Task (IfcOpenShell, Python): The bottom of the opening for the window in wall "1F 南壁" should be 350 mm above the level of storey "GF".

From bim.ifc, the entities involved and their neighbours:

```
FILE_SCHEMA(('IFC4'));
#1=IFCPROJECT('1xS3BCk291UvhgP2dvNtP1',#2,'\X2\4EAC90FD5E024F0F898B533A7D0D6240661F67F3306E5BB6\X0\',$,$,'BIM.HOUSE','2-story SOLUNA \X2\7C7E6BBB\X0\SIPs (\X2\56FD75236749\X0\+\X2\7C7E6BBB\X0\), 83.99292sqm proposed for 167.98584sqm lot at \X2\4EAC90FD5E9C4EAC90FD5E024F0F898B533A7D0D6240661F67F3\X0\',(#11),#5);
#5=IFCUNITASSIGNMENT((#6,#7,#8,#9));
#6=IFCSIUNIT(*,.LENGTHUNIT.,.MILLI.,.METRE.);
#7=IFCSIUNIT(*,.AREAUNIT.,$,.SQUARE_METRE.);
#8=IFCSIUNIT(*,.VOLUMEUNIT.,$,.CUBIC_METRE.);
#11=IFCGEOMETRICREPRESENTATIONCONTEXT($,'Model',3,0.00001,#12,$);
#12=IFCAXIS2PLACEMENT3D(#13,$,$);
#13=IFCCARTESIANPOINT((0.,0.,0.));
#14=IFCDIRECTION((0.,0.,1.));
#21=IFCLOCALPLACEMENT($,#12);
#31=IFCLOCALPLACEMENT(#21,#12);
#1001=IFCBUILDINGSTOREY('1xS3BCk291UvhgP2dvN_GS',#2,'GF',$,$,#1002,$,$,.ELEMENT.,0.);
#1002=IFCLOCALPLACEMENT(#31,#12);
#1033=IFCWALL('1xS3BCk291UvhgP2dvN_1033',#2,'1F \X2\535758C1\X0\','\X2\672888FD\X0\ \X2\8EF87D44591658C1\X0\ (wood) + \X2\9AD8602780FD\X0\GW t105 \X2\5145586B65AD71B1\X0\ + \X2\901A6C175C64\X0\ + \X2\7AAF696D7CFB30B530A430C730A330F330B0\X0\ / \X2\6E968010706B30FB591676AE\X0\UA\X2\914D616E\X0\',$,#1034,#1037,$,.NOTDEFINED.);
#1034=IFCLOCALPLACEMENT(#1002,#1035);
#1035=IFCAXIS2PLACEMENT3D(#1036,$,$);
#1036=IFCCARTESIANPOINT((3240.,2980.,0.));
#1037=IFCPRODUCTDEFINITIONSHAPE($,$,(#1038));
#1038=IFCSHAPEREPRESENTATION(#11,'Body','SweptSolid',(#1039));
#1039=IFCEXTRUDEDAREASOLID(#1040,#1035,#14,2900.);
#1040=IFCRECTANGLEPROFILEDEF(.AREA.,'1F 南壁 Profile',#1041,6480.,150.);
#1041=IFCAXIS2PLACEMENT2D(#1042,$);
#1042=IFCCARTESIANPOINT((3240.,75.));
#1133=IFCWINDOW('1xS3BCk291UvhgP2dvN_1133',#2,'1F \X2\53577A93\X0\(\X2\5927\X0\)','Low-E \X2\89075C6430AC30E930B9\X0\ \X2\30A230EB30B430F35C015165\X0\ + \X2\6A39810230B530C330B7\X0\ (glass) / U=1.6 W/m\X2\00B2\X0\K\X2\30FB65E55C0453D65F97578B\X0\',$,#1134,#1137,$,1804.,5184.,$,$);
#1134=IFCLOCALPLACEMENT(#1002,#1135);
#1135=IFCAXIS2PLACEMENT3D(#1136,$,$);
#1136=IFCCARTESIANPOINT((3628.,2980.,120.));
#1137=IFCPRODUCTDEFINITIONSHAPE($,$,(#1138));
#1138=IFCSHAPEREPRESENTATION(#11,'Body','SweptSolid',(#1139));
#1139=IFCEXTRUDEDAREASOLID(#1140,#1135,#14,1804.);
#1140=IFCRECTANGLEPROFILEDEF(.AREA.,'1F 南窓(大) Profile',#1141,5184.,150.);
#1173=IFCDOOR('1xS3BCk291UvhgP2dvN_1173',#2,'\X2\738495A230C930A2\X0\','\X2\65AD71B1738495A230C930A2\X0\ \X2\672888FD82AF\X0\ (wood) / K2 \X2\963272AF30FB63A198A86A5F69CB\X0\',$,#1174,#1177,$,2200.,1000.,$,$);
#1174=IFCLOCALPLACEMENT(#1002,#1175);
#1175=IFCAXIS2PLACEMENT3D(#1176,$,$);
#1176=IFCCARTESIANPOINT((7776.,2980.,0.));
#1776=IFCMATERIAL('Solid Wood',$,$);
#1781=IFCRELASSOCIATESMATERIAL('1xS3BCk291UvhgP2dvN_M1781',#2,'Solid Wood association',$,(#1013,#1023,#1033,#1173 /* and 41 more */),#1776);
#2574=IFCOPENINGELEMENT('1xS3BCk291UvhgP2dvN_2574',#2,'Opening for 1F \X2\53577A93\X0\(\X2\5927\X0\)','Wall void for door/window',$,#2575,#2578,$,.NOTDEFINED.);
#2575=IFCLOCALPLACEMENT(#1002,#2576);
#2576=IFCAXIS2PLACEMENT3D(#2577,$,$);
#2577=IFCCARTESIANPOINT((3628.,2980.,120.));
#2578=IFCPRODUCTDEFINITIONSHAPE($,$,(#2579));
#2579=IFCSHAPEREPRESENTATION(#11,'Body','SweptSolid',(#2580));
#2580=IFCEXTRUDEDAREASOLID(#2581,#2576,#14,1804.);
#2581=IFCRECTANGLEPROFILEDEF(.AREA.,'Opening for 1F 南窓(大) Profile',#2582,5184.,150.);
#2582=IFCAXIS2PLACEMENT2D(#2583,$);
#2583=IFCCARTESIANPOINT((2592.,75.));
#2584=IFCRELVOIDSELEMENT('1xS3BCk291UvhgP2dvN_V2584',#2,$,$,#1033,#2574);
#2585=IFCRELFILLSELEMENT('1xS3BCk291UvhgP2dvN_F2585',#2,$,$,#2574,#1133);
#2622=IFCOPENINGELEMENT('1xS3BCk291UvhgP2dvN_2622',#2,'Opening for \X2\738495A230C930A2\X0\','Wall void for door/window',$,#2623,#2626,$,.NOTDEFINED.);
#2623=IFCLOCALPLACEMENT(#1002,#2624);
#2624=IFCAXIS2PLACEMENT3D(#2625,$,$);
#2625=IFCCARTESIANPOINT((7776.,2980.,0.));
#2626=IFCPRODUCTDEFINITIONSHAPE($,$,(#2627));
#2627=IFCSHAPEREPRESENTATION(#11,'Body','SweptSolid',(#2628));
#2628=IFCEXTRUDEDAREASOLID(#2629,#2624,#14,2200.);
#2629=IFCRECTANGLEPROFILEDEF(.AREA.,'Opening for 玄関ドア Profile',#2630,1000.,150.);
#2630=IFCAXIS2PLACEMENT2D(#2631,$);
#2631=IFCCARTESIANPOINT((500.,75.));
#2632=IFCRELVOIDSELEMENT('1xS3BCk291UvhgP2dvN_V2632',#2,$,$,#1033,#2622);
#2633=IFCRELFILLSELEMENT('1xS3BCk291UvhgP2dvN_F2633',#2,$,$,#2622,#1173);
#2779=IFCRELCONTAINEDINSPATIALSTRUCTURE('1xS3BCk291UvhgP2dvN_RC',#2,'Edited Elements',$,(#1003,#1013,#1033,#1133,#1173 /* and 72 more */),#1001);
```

```python
import numpy as np
import ifcopenshell
import ifcopenshell.api.geometry
import ifcopenshell.geom
import ifcopenshell.util.element
import ifcopenshell.util.placement
import ifcopenshell.util.shape
import ifcopenshell.util.unit

model = ifcopenshell.open("bim.ifc")
unit_scale = ifcopenshell.util.unit.calculate_unit_scale(model)

window = model.by_guid("1xS3BCk291UvhgP2dvN_1133")
opening = window.FillsVoids[0].RelatingOpeningElement
storey = ifcopenshell.util.element.get_container(window, ifc_class="IfcBuildingStorey")
level = ifcopenshell.util.placement.get_local_placement(storey.ObjectPlacement)[2, 3]

# The opening's origin need not be at the sill, so measure its lowest point.
shape = ifcopenshell.geom.create_shape(ifcopenshell.geom.settings(), opening)
bottom = ifcopenshell.util.shape.get_shape_bottom_elevation(shape, shape.geometry) / unit_scale
dz = level + 350.0 - bottom

shift = np.array([0.0, 0.0, dz])
# The window is not placed relative to its opening, so move both.
for product in (opening, window):
    matrix = ifcopenshell.util.placement.get_local_placement(product.ObjectPlacement)
    matrix[:3, 3] += shift
    ifcopenshell.api.geometry.edit_object_placement(model, product=product, matrix=matrix, is_si=False)

print(f"moved by {dz * unit_scale:+.3f} m")

model.write("bim_edited.ifc")
```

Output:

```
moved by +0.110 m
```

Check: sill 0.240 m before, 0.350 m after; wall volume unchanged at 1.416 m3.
